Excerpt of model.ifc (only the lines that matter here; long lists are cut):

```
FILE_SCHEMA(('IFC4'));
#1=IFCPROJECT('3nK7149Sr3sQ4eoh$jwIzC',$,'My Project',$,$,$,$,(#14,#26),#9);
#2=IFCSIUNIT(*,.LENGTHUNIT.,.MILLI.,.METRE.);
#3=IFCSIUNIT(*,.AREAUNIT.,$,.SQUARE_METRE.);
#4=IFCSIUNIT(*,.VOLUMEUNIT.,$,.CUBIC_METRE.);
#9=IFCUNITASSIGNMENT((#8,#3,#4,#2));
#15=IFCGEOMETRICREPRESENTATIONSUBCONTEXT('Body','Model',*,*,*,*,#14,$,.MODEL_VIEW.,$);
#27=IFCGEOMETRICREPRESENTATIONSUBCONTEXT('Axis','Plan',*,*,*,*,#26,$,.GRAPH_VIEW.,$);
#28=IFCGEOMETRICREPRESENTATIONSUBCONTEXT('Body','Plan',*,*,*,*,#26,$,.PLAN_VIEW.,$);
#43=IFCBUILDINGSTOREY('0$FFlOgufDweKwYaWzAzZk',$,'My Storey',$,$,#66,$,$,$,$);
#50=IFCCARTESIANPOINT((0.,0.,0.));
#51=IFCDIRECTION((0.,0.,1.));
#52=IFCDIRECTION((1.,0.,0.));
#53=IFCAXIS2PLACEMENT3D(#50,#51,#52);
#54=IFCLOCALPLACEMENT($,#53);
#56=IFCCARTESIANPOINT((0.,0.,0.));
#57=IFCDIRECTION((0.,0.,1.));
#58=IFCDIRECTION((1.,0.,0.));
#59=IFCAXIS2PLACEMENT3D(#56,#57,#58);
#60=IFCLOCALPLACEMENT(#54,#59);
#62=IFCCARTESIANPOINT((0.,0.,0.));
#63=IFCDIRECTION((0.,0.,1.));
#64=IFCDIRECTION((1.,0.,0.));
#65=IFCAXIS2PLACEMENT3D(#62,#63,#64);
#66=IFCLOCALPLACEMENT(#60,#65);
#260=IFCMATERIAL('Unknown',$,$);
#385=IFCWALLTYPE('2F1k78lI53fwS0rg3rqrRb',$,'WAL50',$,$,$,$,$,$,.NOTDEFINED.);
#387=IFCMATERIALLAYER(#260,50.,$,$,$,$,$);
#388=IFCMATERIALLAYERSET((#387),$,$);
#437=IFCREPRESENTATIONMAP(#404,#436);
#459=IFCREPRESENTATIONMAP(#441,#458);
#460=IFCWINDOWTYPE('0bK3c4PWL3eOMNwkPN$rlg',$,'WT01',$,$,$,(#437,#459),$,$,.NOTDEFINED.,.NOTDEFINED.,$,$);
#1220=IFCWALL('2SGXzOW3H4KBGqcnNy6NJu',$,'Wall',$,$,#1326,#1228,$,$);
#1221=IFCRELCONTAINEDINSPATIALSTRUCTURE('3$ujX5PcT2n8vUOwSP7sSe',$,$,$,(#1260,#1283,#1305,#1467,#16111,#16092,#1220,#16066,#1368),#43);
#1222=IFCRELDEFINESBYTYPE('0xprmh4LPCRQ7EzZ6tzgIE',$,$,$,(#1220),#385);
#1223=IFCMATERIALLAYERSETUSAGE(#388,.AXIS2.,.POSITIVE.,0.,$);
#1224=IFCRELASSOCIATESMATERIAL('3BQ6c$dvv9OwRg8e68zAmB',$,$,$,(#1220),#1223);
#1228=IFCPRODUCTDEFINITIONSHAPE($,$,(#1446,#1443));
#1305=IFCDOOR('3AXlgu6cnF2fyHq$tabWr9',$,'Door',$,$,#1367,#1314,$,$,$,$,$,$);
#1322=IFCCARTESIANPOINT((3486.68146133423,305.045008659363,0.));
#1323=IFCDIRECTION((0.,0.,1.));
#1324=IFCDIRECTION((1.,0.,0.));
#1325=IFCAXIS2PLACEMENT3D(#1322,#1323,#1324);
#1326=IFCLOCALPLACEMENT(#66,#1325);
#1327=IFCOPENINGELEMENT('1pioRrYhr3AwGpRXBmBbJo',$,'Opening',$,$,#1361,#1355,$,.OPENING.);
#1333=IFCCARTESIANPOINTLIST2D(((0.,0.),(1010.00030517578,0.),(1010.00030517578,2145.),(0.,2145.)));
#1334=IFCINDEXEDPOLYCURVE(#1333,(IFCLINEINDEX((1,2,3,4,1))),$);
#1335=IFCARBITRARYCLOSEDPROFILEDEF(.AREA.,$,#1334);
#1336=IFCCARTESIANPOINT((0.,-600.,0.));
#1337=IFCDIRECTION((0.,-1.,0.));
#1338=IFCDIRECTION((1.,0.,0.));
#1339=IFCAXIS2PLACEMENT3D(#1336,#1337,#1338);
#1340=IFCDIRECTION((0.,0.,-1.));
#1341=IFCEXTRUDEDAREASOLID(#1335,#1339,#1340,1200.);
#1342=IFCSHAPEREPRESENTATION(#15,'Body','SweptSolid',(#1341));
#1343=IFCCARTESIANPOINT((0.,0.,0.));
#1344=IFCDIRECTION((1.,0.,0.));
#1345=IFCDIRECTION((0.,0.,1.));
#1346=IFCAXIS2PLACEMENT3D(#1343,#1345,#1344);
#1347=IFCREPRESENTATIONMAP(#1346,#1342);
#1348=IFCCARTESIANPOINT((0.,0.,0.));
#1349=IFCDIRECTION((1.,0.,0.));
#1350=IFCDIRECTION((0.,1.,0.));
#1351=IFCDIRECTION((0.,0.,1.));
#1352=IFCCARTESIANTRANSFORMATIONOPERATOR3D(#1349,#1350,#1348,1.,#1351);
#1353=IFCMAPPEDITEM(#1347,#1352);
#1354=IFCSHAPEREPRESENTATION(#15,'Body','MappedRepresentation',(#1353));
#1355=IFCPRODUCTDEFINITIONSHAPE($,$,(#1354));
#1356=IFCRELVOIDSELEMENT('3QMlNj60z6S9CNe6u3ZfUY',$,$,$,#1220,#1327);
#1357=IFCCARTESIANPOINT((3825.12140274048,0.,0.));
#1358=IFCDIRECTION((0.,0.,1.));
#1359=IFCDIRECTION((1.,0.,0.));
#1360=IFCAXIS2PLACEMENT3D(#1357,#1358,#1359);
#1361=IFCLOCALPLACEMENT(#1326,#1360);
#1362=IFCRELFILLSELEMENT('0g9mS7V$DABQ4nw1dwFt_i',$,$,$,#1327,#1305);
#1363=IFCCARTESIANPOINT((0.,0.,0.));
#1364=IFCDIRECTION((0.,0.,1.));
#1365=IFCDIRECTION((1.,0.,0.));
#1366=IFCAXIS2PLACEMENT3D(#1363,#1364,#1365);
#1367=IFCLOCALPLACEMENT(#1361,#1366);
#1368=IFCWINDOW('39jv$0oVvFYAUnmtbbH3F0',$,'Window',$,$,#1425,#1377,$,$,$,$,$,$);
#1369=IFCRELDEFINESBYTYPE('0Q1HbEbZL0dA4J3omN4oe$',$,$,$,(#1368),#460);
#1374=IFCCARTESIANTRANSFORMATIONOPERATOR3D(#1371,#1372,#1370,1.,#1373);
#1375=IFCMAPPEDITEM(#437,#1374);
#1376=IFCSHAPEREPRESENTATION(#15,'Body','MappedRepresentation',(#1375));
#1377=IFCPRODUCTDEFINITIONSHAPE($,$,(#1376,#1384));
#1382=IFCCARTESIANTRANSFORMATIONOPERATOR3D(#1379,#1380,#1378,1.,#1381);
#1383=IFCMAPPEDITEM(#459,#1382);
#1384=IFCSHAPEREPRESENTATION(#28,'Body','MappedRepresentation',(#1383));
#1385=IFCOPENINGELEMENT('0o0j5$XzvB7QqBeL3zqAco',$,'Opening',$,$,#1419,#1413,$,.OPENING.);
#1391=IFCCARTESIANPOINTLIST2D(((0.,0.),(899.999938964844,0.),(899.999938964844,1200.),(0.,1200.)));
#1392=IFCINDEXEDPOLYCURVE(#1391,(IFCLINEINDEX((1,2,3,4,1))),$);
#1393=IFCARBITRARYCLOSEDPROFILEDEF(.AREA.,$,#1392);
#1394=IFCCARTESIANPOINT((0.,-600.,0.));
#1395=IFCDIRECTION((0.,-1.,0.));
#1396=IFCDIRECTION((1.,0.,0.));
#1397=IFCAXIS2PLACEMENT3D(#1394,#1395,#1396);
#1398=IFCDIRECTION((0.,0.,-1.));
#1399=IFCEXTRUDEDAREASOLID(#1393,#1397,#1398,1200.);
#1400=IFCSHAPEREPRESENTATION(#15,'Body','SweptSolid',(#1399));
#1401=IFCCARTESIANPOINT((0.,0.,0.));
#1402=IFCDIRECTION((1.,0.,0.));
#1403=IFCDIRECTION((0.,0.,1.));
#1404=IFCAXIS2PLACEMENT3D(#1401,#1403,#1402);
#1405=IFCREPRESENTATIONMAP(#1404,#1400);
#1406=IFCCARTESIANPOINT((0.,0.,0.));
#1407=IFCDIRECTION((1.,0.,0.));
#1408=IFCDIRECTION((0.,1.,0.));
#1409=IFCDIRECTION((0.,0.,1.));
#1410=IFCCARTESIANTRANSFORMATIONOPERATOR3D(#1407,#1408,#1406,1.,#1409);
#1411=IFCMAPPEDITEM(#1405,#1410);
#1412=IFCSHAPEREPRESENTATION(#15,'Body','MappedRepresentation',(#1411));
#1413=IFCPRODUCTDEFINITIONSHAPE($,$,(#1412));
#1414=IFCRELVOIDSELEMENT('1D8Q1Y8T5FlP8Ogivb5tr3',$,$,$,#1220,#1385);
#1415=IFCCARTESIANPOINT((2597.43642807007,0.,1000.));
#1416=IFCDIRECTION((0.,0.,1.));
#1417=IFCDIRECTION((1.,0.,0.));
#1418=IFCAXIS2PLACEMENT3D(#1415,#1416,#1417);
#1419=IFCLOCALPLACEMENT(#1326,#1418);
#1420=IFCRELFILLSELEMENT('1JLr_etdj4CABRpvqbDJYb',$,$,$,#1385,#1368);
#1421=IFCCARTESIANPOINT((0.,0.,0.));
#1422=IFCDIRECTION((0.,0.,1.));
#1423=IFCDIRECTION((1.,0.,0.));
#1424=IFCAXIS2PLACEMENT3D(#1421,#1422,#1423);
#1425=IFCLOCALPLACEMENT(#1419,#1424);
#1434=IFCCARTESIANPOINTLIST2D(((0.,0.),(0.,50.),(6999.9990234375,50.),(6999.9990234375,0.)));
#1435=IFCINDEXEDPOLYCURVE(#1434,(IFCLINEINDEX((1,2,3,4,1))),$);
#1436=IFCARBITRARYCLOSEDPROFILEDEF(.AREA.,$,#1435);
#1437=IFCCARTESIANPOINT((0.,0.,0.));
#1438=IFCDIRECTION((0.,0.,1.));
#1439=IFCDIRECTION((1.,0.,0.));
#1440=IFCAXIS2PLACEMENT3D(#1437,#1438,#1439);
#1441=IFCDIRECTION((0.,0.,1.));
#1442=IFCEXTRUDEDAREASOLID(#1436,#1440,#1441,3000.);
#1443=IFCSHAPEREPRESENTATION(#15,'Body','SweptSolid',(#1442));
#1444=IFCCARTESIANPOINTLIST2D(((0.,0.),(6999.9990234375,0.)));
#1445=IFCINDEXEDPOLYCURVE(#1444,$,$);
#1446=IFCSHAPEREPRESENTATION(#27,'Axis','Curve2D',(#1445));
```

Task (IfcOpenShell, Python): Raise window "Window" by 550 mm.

```python
import numpy as np
import ifcopenshell
import ifcopenshell.api.geometry
import ifcopenshell.util.placement
import ifcopenshell.util.unit

model = ifcopenshell.open("model.ifc")
unit_scale = ifcopenshell.util.unit.calculate_unit_scale(model)

window = model.by_guid("39jv$0oVvFYAUnmtbbH3F0")
opening = window.FillsVoids[0].RelatingOpeningElement
dz = 550.0

shift = np.array([0.0, 0.0, dz])
# The window is placed relative to its opening, so it follows when the opening moves.
matrix = ifcopenshell.util.placement.get_local_placement(opening.ObjectPlacement)
matrix[:3, 3] += shift
ifcopenshell.api.geometry.edit_object_placement(
    model, product=opening, matrix=matrix, is_si=False, should_transform_children=True
)

print(f"moved by {dz * unit_scale:+.3f} m")

model.write("model_updated.ifc")
```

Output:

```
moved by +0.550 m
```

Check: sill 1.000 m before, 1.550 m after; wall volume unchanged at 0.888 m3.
